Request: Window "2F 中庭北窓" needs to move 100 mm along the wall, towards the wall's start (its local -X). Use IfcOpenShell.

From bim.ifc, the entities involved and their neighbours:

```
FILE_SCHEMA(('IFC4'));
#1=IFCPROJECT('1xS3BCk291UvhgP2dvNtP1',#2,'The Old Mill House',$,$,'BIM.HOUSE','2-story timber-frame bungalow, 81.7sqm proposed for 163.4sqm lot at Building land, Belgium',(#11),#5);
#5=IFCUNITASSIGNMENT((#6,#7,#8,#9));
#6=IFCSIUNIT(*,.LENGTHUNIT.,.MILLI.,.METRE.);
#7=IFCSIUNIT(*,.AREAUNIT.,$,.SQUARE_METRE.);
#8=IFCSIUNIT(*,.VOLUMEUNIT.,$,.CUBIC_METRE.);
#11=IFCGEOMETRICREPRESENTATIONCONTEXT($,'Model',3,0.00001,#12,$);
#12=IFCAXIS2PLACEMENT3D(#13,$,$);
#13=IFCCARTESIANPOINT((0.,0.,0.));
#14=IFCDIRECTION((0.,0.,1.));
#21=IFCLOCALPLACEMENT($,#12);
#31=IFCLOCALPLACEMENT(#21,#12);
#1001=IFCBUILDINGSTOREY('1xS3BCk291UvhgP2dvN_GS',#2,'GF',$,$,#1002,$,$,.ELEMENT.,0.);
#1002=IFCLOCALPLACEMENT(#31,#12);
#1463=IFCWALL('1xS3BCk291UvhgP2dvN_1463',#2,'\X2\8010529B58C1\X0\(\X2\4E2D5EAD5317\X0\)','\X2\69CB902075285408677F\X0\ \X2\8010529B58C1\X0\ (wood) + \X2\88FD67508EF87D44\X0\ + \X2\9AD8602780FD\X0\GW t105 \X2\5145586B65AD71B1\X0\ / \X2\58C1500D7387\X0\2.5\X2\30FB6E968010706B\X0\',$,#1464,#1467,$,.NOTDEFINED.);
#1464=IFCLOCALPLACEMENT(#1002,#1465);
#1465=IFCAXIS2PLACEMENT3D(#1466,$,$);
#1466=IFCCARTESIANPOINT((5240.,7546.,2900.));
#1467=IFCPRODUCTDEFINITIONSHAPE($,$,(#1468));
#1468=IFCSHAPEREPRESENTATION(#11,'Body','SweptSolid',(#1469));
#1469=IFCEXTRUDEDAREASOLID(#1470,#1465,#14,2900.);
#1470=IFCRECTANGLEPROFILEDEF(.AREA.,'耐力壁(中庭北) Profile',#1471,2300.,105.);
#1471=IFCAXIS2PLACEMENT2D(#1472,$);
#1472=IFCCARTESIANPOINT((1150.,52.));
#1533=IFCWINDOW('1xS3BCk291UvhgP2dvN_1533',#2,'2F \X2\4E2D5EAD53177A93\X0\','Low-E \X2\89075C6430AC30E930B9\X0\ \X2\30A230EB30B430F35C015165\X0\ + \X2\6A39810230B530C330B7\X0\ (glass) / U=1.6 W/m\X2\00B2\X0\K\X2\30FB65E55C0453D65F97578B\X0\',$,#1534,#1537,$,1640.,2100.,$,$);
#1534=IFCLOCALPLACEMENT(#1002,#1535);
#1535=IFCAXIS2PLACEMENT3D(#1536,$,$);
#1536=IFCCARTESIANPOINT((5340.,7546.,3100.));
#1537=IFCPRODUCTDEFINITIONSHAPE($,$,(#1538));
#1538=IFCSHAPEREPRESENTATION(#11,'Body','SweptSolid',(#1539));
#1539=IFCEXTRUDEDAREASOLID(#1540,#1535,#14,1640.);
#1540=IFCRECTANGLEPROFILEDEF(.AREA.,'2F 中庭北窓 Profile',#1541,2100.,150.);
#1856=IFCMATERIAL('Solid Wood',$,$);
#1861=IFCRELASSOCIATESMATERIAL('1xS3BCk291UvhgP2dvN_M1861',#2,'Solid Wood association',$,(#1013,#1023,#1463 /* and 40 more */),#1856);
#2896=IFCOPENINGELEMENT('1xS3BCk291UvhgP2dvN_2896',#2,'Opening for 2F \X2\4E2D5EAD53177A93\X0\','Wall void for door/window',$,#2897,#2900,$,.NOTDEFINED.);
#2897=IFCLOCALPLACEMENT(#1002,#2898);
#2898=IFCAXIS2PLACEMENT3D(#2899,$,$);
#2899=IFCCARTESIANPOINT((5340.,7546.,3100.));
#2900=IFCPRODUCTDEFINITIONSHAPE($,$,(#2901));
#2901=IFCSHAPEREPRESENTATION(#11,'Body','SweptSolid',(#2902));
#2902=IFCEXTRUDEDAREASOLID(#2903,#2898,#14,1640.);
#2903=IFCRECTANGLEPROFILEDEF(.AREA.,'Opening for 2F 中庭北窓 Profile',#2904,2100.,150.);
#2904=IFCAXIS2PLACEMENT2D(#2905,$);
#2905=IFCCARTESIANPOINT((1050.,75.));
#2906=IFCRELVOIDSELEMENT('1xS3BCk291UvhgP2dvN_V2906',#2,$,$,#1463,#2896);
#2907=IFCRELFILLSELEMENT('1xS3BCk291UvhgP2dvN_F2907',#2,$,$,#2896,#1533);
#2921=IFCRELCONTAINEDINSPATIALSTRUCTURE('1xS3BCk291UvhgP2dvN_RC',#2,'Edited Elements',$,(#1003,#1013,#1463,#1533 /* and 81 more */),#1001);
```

```python
import ifcopenshell
import ifcopenshell.api.geometry
import ifcopenshell.util.placement
import ifcopenshell.util.unit

model = ifcopenshell.open("bim.ifc")
unit_scale = ifcopenshell.util.unit.calculate_unit_scale(model)

window = model.by_id(1533)
opening = window.FillsVoids[0].RelatingOpeningElement
wall = opening.VoidsElements[0].RelatingBuildingElement

wall_matrix = ifcopenshell.util.placement.get_local_placement(wall.ObjectPlacement)
shift = wall_matrix[:3, 0] * -0.1 / unit_scale
before = ifcopenshell.util.placement.get_local_placement(window.ObjectPlacement)[:3, 3].copy()

# The window is not placed relative to its opening, so move both.
for product in (opening, window):
    matrix = ifcopenshell.util.placement.get_local_placement(product.ObjectPlacement)
    matrix[:3, 3] += shift
    ifcopenshell.api.geometry.edit_object_placement(model, product=product, matrix=matrix, is_si=False)

after = ifcopenshell.util.placement.get_local_placement(window.ObjectPlacement)[:3, 3]
print("window moved by", (after - before).round(3) + 0.0)

model.write("bim_rev.ifc")
```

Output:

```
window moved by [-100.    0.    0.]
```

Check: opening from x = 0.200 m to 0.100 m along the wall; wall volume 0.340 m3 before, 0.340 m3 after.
